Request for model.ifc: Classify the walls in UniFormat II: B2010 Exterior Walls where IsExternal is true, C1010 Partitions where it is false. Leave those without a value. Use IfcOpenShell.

First a look at what the model holds.

```python
import ifcopenshell
import ifcopenshell.util.element

model = ifcopenshell.open("model.ifc")
print(model.schema)
print("classifications:", [c.Name for c in model.by_type("IfcClassification")])
values = [ifcopenshell.util.element.get_pset(e, "Pset_WallCommon", "IsExternal") for e in model.by_type("IfcWall")]
for value in (True, False, None):
    print("IsExternal", value, values.count(value))
```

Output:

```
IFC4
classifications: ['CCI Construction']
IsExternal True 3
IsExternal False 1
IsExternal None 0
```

```python
import ifcopenshell
import ifcopenshell.api.classification
import ifcopenshell.util.element

model = ifcopenshell.open("model.ifc")

system = ifcopenshell.api.classification.add_classification(model, classification="UniFormat II")

walls = model.by_type("IfcWall")
external = {e: ifcopenshell.util.element.get_pset(e, "Pset_WallCommon", "IsExternal") for e in walls}
for flag, code, name in ((True, "B2010", "Exterior Walls"), (False, "C1010", "Partitions")):
    products = [e for e in walls if external[e] is flag]
    ifcopenshell.api.classification.add_reference(
        model, products=products, classification=system, identification=code, name=name
    )
    print(code, len(products))

model.write("model_rev.ifc")
```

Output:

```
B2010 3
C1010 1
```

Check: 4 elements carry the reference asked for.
